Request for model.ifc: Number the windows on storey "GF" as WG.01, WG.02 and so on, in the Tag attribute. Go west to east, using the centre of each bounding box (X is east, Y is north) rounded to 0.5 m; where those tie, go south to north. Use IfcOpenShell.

First a look at what the model holds.

```python
import ifcopenshell
import ifcopenshell.util.element
import ifcopenshell.util.placement

model = ifcopenshell.open("model.ifc")
print(model.schema)
storey = next(s for s in model.by_type("IfcBuildingStorey") if s.Name == "GF")
windows = [e for e in ifcopenshell.util.element.get_decomposition(storey) if e.is_a("IfcWindow")]
for e in sorted(windows, key=lambda e: e.id()):
    origin = ifcopenshell.util.placement.get_local_placement(e.ObjectPlacement)[:3, 3]
    print(e.id(), e.Tag, e.Name, origin.round(2) + 0.0, sep=" | ")
```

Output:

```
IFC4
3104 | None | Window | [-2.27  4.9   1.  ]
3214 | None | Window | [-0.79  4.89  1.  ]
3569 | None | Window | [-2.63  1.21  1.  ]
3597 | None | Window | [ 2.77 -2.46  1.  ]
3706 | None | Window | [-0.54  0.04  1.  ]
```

```python
import ifcopenshell
import ifcopenshell.geom
import ifcopenshell.util.element
import ifcopenshell.util.shape

model = ifcopenshell.open("model.ifc")
settings = ifcopenshell.geom.settings()
settings.set("use-world-coords", True)


def centre(element):
    shape = ifcopenshell.geom.create_shape(settings, element)
    return ifcopenshell.util.shape.get_bbox_centroid(shape.geometry)


storey = next(s for s in model.by_type("IfcBuildingStorey") if s.Name == "GF")
windows = [e for e in ifcopenshell.util.element.get_decomposition(storey) if e.is_a("IfcWindow")]

# Insertion points can sit at a corner or the storey origin, so sort by the geometry (in metres).
centres = {e: centre(e) for e in windows}
windows.sort(key=lambda e: (round(centres[e][0] / 0.5), centres[e][1]))

for i, e in enumerate(windows, start=1):
    number = f"WG.{i:02d}"
    e.Tag = number
    print(e.id(), number)

model.write("model_rev.ifc")
```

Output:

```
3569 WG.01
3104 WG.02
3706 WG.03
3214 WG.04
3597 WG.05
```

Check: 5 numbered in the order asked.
